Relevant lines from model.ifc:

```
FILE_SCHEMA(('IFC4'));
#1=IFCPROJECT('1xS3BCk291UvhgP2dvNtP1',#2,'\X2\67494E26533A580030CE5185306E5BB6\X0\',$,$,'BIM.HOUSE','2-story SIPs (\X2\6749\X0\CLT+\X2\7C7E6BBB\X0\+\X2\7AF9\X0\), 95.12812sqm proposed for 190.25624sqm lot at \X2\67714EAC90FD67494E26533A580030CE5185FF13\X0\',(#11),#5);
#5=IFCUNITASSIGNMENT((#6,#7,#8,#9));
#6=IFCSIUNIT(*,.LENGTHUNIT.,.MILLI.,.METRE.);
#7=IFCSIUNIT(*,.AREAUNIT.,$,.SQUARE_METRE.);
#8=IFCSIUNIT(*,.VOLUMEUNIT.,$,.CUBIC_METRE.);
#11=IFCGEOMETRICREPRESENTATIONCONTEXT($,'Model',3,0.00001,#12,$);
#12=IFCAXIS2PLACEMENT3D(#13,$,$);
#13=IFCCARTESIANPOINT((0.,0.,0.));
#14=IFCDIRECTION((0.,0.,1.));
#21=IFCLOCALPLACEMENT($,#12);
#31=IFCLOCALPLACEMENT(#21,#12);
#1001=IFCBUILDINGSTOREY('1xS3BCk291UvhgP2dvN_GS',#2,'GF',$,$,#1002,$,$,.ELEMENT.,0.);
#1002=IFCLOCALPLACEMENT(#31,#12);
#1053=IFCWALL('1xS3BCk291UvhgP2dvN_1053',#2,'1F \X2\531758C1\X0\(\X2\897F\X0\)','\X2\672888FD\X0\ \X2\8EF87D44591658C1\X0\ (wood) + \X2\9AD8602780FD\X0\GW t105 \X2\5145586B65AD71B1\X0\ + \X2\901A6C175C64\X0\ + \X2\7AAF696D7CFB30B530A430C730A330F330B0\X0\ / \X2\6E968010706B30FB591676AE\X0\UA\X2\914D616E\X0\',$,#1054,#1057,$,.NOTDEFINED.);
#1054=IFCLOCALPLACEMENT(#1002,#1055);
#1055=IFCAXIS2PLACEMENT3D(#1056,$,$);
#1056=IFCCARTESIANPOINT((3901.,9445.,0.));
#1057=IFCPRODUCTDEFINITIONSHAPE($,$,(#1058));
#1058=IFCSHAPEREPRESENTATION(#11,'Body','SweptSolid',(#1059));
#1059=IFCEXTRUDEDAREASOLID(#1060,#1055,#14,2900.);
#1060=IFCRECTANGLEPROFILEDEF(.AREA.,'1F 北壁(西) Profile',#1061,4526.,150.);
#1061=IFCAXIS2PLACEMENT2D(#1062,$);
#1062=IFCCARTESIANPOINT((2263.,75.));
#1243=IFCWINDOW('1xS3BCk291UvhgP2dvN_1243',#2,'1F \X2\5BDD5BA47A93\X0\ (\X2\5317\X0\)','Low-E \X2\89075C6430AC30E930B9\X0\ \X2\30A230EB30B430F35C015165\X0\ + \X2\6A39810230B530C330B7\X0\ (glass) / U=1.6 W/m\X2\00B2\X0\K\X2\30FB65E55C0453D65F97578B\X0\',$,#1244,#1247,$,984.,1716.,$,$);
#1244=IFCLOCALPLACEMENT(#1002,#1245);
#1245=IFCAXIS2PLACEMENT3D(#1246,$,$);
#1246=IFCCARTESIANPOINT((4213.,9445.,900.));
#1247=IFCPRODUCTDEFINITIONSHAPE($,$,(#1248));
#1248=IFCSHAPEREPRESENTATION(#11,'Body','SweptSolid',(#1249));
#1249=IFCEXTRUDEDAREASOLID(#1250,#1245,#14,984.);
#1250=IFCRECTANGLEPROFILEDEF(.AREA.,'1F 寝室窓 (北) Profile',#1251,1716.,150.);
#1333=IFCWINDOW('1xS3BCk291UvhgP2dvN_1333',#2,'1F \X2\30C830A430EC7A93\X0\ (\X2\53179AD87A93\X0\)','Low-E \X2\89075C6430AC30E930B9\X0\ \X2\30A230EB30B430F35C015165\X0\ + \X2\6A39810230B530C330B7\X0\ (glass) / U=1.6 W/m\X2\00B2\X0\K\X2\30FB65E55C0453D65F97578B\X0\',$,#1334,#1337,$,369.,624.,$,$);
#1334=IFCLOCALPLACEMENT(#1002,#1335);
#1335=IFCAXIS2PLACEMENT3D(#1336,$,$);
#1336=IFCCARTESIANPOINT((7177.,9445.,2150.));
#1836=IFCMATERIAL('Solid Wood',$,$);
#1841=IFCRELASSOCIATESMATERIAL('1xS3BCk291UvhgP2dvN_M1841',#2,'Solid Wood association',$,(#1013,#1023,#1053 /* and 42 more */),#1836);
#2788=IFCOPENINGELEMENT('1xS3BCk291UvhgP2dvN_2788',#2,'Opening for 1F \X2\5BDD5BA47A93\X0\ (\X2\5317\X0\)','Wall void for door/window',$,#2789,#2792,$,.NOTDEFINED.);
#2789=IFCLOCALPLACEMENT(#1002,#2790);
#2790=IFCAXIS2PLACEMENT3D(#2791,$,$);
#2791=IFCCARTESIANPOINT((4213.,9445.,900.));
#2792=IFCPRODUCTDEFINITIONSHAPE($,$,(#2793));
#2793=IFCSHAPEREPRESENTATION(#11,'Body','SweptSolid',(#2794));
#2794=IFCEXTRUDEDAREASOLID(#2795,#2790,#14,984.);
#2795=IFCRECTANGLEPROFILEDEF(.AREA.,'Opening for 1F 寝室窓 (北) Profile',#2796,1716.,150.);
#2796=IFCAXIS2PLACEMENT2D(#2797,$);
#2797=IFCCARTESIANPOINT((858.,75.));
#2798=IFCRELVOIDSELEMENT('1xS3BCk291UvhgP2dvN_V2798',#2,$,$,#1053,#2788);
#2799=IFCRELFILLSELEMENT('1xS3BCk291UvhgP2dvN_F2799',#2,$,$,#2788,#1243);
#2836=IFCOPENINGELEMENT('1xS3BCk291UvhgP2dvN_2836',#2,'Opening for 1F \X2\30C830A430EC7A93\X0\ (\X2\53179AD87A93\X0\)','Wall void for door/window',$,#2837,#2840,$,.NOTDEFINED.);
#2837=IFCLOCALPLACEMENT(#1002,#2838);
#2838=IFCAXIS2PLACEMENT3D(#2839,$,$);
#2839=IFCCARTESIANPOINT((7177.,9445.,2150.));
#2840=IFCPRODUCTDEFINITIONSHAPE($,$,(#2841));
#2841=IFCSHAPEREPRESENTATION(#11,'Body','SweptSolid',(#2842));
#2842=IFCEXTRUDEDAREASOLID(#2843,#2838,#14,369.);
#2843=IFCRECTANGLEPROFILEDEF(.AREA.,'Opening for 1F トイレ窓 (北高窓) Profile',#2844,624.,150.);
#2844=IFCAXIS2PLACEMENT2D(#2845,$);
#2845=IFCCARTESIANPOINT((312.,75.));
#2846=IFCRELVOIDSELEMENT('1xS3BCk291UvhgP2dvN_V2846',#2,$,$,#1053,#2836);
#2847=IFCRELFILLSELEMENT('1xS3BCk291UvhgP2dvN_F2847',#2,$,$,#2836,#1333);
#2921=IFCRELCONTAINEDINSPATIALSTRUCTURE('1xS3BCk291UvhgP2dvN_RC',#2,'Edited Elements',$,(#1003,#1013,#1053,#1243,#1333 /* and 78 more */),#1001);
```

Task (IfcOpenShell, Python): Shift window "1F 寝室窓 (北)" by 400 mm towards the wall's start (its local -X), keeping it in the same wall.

```python
import ifcopenshell
import ifcopenshell.api.geometry
import ifcopenshell.util.placement

model = ifcopenshell.open("model.ifc")

window = model.by_guid("1xS3BCk291UvhgP2dvN_1243")
opening = window.FillsVoids[0].RelatingOpeningElement
wall = opening.VoidsElements[0].RelatingBuildingElement

wall_matrix = ifcopenshell.util.placement.get_local_placement(wall.ObjectPlacement)
shift = wall_matrix[:3, 0] * -400.0
before = ifcopenshell.util.placement.get_local_placement(window.ObjectPlacement)[:3, 3].copy()

# The window is not placed relative to its opening, so move both.
for product in (opening, window):
    matrix = ifcopenshell.util.placement.get_local_placement(product.ObjectPlacement)
    matrix[:3, 3] += shift
    ifcopenshell.api.geometry.edit_object_placement(model, product=product, matrix=matrix, is_si=False)

after = ifcopenshell.util.placement.get_local_placement(window.ObjectPlacement)[:3, 3]
print("window moved by", (after - before).round(3) + 0.0)

model.write("model_rev.ifc")
```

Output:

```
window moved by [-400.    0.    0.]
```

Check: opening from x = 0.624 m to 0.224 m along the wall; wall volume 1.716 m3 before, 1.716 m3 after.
